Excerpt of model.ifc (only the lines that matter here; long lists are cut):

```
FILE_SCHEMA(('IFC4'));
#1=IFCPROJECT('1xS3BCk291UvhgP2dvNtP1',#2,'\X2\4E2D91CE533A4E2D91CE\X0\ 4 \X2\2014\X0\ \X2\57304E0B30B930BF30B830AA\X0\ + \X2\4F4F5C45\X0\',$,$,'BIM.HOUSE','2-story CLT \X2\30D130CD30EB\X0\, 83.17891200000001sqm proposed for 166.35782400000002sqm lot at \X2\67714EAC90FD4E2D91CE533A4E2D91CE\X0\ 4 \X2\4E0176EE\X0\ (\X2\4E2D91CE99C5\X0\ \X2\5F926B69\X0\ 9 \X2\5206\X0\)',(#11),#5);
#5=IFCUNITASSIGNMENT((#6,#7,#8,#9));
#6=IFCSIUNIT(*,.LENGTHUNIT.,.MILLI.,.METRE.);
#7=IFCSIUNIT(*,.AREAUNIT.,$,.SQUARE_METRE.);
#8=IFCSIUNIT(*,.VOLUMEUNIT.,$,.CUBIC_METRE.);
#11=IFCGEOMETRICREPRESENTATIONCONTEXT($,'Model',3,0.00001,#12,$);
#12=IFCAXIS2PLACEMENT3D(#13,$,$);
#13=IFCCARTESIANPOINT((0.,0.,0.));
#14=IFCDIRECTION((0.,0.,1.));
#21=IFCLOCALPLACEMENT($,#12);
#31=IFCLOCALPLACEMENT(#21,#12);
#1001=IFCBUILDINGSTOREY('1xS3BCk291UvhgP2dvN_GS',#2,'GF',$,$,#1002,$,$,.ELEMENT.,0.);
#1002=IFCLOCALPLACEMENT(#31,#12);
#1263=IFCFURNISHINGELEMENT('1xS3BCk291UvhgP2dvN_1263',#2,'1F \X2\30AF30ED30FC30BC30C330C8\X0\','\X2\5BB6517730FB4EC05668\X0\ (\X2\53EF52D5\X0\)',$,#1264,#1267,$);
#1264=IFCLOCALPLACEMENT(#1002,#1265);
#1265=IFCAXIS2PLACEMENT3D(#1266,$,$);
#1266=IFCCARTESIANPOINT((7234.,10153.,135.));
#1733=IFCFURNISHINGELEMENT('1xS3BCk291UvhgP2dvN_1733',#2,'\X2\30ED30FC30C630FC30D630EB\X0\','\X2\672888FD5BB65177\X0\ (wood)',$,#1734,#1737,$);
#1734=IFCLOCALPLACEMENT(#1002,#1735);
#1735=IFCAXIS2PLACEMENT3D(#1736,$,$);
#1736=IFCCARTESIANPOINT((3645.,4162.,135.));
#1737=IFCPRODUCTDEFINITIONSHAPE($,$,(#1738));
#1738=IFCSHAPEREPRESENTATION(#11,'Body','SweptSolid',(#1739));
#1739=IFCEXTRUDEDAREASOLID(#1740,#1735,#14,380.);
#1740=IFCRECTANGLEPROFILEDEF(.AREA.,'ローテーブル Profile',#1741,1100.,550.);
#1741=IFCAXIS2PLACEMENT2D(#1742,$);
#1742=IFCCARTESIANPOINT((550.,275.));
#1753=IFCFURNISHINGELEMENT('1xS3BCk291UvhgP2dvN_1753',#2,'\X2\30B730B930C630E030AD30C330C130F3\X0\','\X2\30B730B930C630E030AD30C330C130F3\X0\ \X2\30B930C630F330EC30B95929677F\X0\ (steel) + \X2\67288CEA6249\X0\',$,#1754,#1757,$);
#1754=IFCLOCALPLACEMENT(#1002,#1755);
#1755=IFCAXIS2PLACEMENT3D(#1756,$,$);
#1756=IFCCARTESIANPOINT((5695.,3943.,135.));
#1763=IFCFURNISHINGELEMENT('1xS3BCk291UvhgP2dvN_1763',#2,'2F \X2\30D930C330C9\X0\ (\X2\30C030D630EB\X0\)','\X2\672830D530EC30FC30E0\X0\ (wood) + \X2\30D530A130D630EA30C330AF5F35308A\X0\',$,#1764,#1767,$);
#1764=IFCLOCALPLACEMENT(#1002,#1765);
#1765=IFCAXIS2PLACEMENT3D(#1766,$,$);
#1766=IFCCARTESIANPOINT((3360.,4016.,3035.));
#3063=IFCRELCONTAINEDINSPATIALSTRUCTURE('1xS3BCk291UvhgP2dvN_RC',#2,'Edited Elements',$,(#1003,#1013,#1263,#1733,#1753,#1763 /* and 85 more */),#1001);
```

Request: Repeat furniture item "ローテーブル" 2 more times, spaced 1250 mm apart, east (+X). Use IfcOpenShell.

```python
import numpy as np
import ifcopenshell
import ifcopenshell.api.geometry
import ifcopenshell.api.root
import ifcopenshell.util.element
import ifcopenshell.util.placement

model = ifcopenshell.open("model.ifc")


def reuse_history(source, copy):
    """copy_class also copies each property set's owner history, people and application; keep the originals."""
    for rel in copy.IsDefinedBy:
        if rel.is_a("IfcRelDefinesByProperties") and (history := rel.RelatingPropertyDefinition.OwnerHistory):
            rel.RelatingPropertyDefinition.OwnerHistory = source.OwnerHistory
            ifcopenshell.util.element.remove_deep2(model, history)


source = model.by_guid("1xS3BCk291UvhgP2dvN_1733")
base = ifcopenshell.util.placement.get_local_placement(source.ObjectPlacement)
step = np.array([1.0, 0.0, 0.0]) * 1250.0

for i in range(1, 3):
    copy = ifcopenshell.api.root.copy_class(model, product=source)
    copy.Representation = ifcopenshell.util.element.copy_deep(
        model, source.Representation, exclude=["IfcGeometricRepresentationContext", "IfcRepresentationMap"]
    )
    reuse_history(source, copy)
    matrix = base.copy()
    matrix[:3, 3] += i * step
    print("added at", matrix[:3, 3].round(3) + 0.0)
    ifcopenshell.api.geometry.edit_object_placement(model, product=copy, matrix=matrix, is_si=False)

model.write("model_updated.ifc")
```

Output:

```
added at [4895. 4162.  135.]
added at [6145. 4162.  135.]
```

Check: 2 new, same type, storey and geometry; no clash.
